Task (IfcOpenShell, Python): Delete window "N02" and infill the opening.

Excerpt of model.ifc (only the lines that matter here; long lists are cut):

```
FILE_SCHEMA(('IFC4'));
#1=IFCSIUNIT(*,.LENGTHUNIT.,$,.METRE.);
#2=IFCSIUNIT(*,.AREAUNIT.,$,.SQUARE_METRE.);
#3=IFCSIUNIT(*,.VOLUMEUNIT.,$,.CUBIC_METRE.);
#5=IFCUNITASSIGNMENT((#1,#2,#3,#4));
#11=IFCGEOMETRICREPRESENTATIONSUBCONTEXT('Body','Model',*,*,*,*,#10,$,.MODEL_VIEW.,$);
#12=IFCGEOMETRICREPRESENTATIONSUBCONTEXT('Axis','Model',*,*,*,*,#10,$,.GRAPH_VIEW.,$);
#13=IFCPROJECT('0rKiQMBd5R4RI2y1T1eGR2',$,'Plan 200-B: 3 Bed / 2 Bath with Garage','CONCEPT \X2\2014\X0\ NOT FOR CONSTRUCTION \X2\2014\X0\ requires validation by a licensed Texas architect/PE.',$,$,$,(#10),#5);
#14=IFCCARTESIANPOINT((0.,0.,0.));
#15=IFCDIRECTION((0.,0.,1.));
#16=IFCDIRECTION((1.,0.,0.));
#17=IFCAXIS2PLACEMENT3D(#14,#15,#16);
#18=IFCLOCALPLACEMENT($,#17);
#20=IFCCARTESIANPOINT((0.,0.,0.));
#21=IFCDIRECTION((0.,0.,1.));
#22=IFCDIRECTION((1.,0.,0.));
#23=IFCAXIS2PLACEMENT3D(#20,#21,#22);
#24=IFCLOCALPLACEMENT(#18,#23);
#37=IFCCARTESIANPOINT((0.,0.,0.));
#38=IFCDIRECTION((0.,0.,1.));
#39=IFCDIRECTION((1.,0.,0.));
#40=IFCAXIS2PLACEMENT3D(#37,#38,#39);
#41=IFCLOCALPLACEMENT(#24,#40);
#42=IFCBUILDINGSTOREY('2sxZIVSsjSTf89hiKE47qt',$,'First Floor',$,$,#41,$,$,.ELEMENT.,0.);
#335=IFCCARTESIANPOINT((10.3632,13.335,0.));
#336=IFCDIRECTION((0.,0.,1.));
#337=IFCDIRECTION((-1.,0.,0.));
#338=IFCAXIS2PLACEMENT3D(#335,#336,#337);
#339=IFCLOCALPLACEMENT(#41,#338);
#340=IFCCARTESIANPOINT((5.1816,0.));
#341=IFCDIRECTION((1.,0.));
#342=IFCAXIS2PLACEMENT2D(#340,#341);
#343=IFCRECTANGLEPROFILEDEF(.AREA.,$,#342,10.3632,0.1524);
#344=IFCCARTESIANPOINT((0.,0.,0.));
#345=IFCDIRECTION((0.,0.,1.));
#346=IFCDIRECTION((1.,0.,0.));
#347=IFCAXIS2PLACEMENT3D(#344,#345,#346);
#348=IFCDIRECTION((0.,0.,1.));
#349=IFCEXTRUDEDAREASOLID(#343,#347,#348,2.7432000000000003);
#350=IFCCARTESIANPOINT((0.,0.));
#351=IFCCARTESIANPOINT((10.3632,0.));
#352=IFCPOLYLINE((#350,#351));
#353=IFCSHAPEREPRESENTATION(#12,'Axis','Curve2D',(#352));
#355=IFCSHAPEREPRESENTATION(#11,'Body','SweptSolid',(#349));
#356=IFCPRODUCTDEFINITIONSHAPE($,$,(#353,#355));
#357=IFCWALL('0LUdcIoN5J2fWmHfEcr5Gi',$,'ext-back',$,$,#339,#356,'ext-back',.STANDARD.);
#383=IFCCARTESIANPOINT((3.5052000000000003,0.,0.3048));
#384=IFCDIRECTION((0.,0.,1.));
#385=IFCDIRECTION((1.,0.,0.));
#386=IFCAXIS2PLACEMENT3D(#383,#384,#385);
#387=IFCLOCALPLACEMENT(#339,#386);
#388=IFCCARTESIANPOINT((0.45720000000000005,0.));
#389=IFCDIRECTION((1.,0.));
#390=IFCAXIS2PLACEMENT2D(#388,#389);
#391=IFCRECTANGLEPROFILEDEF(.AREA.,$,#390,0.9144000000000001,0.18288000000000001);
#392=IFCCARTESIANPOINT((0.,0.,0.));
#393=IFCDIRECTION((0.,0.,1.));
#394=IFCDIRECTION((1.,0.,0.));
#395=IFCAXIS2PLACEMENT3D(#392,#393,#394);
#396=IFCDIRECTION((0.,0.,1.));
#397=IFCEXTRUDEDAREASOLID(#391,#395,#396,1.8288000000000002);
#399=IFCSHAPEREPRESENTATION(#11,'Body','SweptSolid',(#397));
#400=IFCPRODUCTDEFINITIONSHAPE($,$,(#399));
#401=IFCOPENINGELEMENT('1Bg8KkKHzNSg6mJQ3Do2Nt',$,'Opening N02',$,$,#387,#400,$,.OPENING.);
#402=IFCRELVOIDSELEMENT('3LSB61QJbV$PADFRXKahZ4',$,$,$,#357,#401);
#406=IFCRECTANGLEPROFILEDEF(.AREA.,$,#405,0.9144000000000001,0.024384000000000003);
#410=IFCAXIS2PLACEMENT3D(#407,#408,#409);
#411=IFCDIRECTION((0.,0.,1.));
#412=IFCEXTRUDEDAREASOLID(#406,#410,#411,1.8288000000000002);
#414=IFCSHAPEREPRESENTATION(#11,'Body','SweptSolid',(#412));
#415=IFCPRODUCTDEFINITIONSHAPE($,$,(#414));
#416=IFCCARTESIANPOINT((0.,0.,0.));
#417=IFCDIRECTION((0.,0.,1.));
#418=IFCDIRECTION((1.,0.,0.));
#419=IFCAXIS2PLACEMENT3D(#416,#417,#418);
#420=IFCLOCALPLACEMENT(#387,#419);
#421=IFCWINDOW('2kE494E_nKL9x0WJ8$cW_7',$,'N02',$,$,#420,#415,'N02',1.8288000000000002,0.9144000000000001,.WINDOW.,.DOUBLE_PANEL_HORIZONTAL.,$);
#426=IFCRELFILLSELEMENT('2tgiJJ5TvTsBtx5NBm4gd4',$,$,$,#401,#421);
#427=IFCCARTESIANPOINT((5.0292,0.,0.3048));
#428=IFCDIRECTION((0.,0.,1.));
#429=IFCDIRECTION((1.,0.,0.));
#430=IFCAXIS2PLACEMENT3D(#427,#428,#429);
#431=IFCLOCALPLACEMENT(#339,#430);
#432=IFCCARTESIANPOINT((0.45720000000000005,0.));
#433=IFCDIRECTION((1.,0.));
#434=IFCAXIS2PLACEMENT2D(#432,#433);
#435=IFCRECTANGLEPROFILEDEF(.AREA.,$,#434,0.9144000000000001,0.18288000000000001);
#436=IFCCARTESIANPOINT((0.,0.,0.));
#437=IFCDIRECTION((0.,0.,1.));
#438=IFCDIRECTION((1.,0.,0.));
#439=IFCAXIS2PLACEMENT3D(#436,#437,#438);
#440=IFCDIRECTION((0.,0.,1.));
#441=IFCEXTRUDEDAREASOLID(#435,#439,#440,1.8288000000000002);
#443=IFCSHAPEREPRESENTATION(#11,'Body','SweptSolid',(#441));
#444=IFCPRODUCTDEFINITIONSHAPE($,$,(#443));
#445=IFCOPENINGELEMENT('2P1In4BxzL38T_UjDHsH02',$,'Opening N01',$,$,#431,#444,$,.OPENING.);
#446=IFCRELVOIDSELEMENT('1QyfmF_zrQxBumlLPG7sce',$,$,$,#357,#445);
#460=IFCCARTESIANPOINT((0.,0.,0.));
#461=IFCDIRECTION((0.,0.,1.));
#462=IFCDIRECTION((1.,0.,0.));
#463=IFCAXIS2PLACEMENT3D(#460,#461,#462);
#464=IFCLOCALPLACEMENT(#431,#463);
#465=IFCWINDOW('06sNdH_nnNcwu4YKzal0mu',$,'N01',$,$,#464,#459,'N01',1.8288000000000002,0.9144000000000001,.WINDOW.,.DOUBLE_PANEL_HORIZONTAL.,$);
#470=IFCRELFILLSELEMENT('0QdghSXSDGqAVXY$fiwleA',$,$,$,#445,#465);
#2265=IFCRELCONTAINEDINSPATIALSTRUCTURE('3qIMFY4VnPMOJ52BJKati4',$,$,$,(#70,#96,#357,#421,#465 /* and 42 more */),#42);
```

```python
import ifcopenshell
import ifcopenshell.api.feature
import ifcopenshell.api.root
import ifcopenshell.geom
import ifcopenshell.util.shape

model = ifcopenshell.open("model.ifc")
settings = ifcopenshell.geom.settings()


def volume(element):
    """Net volume in cubic metres, openings subtracted."""
    shape = ifcopenshell.geom.create_shape(settings, element)
    return ifcopenshell.util.shape.get_volume(shape.geometry)


window = model.by_guid("2kE494E_nKL9x0WJ8$cW_7")
opening = window.FillsVoids[0].RelatingOpeningElement
wall = opening.VoidsElements[0].RelatingBuildingElement
before = volume(wall)

ifcopenshell.api.root.remove_product(model, product=window)
ifcopenshell.api.feature.remove_feature(model, feature=opening)

after = volume(wall)

print(f"wall volume {before:.3f} -> {after:.3f} m3")

model.write("model_updated.ifc")
```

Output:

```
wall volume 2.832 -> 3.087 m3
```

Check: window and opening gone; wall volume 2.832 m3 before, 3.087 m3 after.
